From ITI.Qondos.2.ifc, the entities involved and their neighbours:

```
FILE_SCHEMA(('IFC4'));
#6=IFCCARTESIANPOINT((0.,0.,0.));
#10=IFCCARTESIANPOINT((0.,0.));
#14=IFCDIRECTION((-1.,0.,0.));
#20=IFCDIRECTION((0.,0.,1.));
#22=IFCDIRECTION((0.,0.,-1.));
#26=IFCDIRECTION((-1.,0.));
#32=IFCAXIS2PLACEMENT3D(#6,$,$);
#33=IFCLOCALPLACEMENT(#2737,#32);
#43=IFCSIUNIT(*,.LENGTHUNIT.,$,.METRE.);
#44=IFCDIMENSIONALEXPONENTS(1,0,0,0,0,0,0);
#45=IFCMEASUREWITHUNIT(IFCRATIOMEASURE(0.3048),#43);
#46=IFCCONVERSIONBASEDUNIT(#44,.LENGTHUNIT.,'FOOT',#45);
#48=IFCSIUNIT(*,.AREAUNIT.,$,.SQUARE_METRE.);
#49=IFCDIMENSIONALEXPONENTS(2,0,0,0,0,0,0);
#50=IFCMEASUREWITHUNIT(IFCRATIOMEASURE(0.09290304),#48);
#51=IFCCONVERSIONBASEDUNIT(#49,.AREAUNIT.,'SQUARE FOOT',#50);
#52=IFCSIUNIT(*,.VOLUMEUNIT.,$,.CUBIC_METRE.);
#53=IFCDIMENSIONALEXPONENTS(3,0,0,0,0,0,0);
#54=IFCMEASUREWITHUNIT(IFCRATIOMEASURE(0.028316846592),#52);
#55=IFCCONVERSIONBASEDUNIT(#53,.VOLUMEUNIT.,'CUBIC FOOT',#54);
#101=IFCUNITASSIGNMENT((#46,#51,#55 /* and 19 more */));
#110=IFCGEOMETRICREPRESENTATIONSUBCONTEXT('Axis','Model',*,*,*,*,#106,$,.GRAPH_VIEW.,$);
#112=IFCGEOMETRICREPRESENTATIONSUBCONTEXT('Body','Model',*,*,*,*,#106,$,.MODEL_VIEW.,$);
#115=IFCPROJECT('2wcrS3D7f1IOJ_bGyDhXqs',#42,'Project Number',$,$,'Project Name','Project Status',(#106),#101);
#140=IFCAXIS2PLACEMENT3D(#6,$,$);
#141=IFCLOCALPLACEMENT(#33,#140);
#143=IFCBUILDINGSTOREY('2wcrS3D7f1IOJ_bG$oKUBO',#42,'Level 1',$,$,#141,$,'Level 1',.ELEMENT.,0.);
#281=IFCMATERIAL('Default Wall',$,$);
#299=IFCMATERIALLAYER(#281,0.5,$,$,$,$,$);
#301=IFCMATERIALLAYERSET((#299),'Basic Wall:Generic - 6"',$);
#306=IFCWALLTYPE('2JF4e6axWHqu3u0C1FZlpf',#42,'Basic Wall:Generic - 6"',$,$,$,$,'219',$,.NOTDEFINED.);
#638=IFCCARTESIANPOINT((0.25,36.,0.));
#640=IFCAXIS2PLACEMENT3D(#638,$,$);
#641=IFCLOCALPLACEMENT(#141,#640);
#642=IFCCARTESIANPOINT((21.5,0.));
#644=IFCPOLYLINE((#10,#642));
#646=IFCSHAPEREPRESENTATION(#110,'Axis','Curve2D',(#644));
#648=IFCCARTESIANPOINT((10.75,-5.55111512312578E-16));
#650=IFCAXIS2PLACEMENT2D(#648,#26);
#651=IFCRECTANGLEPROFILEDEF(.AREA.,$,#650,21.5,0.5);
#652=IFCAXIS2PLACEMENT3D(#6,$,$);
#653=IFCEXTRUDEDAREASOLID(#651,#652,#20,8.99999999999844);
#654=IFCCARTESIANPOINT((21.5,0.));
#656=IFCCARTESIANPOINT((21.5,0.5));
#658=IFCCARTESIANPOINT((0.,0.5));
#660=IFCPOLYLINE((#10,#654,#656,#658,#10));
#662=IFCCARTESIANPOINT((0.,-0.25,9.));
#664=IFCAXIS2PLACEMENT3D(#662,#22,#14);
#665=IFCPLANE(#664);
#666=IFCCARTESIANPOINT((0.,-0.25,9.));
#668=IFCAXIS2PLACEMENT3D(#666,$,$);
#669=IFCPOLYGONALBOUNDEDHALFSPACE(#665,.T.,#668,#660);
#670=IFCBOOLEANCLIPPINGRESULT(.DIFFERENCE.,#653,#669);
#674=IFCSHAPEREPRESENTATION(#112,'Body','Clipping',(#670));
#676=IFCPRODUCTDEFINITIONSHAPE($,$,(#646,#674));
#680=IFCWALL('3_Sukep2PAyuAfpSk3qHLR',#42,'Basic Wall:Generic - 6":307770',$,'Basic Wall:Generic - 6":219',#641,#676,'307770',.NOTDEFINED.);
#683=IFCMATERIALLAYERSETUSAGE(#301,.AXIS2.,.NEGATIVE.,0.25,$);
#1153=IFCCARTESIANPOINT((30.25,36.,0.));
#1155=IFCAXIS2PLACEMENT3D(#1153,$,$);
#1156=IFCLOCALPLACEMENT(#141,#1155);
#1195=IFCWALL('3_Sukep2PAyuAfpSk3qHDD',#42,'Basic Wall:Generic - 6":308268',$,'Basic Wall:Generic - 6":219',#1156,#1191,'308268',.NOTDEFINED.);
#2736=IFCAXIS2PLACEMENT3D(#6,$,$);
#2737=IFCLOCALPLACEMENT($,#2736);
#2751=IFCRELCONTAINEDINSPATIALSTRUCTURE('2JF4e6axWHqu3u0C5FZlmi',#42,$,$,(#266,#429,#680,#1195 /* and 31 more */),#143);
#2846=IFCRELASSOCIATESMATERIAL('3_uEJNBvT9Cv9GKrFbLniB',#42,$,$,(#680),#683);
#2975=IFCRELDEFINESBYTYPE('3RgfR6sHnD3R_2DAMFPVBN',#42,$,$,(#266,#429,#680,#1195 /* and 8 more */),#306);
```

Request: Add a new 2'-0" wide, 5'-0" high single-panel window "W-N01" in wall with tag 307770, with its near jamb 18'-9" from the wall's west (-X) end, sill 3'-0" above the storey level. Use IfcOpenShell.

```python
import numpy as np
import ifcopenshell
import ifcopenshell.api.feature
import ifcopenshell.api.geometry
import ifcopenshell.api.root
import ifcopenshell.api.spatial
import ifcopenshell.geom
import ifcopenshell.util.element
import ifcopenshell.util.placement
import ifcopenshell.util.representation
import ifcopenshell.util.shape
import ifcopenshell.util.unit

model = ifcopenshell.open("ITI.Qondos.2.ifc")
unit_scale = ifcopenshell.util.unit.calculate_unit_scale(model)
settings = ifcopenshell.geom.settings()


def volume(element):
    """Net volume in cubic metres, openings subtracted."""
    shape = ifcopenshell.geom.create_shape(settings, element)
    return ifcopenshell.util.shape.get_volume(shape.geometry)


wall = model.by_guid("3_Sukep2PAyuAfpSk3qHLR")
storey = ifcopenshell.util.element.get_container(wall, ifc_class="IfcBuildingStorey")
context = ifcopenshell.util.representation.get_context(model, "Model", "Body", "MODEL_VIEW")
before = volume(wall)

width, height, from_end, sill = 0.6096, 1.524, 5.715, 0.9144  # metres

# The wall runs along its own X axis, and the end named is its -X end.
wall_shape = ifcopenshell.geom.create_shape(settings, wall)
x, y, z = ifcopenshell.util.shape.get_vertices(wall_shape.geometry).T
start = x.min() + from_end
face, thickness = float(y.min()), float(y.max() - y.min())
wall_matrix = ifcopenshell.util.placement.get_local_placement(wall.ObjectPlacement)
level = ifcopenshell.util.placement.get_local_placement(storey.ObjectPlacement)[2, 3]


def in_wall(x, y):
    """Placement at x, y metres in the wall's axes, at sill height."""
    matrix = wall_matrix.copy()
    matrix[:, 3] = wall_matrix @ np.array([x / unit_scale, y / unit_scale, 0.0, 1.0])
    matrix[2, 3] = level + sill / unit_scale
    return matrix


# Opening: a box that overshoots both wall faces by 50 mm.
opening = ifcopenshell.api.root.create_entity(model, ifc_class="IfcOpeningElement", predefined_type="OPENING")
box = ifcopenshell.api.geometry.add_wall_representation(
    model, context=context, length=width, height=height, thickness=thickness + 0.1
)
ifcopenshell.api.geometry.assign_representation(model, product=opening, representation=box)
ifcopenshell.api.geometry.edit_object_placement(model, product=opening, matrix=in_wall(start, face - 0.05), is_si=False)
ifcopenshell.api.feature.add_feature(model, feature=opening, element=wall)

window = ifcopenshell.api.root.create_entity(model, ifc_class="IfcWindow", name="W-N01", predefined_type="WINDOW")
window.OverallWidth, window.OverallHeight = width / unit_scale, height / unit_scale
window.PartitioningType = "SINGLE_PANEL"
body = ifcopenshell.api.geometry.add_window_representation(
    model,
    context=context,
    overall_width=window.OverallWidth,
    overall_height=window.OverallHeight,
    partition_type="SINGLE_PANEL",
)
ifcopenshell.api.geometry.assign_representation(model, product=window, representation=body)
ifcopenshell.api.spatial.assign_container(model, products=[window], relating_structure=storey)
ifcopenshell.api.feature.add_filling(model, opening=opening, element=window)

# Centre the window in the wall's thickness.
ifcopenshell.api.geometry.edit_object_placement(model, product=window, matrix=in_wall(start, face), is_si=False)
window_shape = ifcopenshell.geom.create_shape(settings, window)
depth = ifcopenshell.util.shape.get_vertices(window_shape.geometry)[:, 1]
offset = face + thickness / 2 - (depth.min() + depth.max()) / 2
ifcopenshell.api.geometry.edit_object_placement(model, product=window, matrix=in_wall(start, offset), is_si=False)

after = volume(wall)

print(f"wall volume {before:.3f} -> {after:.3f} m3")

model.write("ITI.Qondos.2_v2.ifc")
```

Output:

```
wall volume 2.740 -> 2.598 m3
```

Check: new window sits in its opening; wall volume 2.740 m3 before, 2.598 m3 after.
